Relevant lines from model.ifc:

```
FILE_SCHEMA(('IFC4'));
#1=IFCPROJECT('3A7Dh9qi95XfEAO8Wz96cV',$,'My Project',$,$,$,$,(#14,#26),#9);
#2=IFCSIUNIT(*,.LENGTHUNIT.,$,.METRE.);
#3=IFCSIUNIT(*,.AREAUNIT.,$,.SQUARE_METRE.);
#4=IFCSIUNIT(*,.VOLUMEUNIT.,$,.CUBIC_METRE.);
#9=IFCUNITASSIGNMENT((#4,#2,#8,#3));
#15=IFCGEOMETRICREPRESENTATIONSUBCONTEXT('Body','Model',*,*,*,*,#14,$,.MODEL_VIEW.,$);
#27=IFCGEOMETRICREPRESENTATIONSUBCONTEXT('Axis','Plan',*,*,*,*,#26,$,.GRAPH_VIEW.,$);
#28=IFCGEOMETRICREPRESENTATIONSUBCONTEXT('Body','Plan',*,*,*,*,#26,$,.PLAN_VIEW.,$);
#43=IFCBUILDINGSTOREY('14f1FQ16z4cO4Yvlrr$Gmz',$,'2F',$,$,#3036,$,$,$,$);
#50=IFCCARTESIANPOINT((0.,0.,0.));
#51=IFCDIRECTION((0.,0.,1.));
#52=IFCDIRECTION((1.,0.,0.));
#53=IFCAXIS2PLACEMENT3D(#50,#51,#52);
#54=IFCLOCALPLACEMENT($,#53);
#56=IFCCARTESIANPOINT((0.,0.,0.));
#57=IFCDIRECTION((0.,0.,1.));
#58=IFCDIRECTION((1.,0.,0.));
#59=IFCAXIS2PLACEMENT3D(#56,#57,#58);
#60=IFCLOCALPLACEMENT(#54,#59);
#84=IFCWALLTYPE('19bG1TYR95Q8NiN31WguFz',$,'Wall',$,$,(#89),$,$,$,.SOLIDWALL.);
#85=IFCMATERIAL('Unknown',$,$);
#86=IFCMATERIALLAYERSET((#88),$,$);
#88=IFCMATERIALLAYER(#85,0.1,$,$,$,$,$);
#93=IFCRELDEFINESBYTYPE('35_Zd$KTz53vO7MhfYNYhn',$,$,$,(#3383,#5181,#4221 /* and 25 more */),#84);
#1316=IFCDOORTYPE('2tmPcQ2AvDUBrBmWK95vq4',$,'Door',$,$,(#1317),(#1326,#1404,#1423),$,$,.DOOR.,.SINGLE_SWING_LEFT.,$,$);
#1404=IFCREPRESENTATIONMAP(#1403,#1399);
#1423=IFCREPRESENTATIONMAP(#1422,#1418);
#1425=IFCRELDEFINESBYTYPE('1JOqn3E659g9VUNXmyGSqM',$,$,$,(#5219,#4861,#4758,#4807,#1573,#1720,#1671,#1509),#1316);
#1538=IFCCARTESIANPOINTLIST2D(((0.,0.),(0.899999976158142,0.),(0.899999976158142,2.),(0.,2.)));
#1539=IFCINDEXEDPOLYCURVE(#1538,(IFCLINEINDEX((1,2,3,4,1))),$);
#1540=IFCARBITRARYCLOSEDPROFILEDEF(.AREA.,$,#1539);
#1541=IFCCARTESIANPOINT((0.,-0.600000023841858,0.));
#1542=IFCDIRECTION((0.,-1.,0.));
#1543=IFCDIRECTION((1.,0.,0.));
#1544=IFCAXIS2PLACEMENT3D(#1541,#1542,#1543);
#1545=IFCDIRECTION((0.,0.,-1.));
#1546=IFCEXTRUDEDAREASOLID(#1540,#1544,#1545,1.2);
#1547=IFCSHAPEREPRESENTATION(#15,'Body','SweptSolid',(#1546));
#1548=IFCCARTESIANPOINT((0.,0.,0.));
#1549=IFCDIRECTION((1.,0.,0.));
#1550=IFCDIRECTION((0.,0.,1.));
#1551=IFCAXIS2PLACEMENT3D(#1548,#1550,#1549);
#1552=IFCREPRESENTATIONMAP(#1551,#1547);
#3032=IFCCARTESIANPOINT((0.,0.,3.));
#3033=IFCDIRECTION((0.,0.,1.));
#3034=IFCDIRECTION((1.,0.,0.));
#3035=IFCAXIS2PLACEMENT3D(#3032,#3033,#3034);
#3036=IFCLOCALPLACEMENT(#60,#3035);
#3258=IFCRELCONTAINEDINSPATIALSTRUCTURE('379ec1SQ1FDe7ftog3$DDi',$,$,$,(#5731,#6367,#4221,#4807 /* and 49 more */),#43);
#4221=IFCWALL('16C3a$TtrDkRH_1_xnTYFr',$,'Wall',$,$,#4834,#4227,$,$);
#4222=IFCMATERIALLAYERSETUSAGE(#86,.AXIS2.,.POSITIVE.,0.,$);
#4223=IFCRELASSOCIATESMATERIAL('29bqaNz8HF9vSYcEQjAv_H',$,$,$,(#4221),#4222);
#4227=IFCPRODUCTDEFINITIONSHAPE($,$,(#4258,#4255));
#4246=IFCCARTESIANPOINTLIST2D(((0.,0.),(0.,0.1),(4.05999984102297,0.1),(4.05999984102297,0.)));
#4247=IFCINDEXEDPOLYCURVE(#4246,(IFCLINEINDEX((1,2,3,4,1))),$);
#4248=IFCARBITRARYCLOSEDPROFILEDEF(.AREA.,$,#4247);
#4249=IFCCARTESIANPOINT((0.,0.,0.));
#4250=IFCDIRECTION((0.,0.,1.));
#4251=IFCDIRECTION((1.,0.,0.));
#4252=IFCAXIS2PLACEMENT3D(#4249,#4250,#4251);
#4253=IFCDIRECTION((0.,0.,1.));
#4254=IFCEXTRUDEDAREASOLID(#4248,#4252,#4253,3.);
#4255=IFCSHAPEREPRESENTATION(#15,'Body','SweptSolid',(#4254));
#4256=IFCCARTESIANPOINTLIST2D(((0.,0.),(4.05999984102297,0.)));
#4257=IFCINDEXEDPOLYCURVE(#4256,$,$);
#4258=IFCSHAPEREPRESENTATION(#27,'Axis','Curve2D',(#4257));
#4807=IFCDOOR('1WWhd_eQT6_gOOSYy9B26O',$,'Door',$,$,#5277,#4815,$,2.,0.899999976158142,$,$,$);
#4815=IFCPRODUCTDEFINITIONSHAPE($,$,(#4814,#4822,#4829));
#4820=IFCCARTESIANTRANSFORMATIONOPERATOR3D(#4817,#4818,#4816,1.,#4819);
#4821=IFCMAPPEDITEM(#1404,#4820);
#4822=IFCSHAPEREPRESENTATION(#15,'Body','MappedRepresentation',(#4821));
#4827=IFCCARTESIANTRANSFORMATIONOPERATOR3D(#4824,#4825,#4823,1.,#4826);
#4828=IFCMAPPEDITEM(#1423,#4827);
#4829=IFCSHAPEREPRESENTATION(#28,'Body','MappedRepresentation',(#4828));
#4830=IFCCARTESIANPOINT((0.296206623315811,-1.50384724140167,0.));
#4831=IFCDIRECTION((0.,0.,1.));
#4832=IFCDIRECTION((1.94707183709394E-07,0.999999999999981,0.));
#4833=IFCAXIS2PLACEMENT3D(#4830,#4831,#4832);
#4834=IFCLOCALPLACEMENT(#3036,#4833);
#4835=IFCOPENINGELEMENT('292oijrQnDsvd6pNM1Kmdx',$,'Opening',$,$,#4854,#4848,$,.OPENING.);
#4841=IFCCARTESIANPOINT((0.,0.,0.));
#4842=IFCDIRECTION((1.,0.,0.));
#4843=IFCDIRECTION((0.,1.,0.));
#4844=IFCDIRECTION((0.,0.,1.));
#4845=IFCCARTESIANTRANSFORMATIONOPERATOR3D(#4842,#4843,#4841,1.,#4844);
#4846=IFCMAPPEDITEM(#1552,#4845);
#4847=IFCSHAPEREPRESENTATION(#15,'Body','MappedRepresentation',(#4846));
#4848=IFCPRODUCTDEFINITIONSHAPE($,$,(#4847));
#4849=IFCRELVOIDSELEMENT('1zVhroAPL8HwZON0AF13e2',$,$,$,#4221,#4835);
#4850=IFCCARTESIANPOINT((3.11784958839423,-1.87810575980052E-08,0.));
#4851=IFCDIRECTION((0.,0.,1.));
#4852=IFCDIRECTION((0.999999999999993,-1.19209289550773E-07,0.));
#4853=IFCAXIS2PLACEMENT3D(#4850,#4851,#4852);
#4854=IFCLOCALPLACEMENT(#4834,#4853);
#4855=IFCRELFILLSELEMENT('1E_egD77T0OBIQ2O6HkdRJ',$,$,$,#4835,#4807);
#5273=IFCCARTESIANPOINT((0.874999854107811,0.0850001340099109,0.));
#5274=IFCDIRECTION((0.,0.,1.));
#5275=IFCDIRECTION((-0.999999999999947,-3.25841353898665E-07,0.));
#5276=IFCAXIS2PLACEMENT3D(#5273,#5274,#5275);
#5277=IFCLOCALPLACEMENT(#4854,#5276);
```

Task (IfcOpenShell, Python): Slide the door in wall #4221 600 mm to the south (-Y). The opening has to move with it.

```python
import ifcopenshell
import ifcopenshell.api.geometry
import ifcopenshell.util.placement

model = ifcopenshell.open("model.ifc")

door = model.by_guid("1WWhd_eQT6_gOOSYy9B26O")
opening = door.FillsVoids[0].RelatingOpeningElement
wall = opening.VoidsElements[0].RelatingBuildingElement

wall_matrix = ifcopenshell.util.placement.get_local_placement(wall.ObjectPlacement)
shift = wall_matrix[:3, 0] * -0.6
before = ifcopenshell.util.placement.get_local_placement(door.ObjectPlacement)[:3, 3].copy()

# The door is placed relative to its opening, so it follows when the opening moves.
matrix = ifcopenshell.util.placement.get_local_placement(opening.ObjectPlacement)
matrix[:3, 3] += shift
ifcopenshell.api.geometry.edit_object_placement(
    model, product=opening, matrix=matrix, is_si=False, should_transform_children=True
)

after = ifcopenshell.util.placement.get_local_placement(door.ObjectPlacement)[:3, 3]
print("door moved by", (after - before).round(3) + 0.0)

model.write("model_rev.ifc")
```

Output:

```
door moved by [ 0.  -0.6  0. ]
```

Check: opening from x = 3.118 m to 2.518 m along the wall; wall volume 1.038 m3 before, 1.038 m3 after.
